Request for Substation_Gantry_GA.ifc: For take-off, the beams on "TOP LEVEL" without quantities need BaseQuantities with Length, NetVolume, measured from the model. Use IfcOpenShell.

First a look at what the model holds.

```python
import ifcopenshell
import ifcopenshell.util.element
import ifcopenshell.util.unit

model = ifcopenshell.open("Substation_Gantry_GA.ifc")
print(model.schema)
for unit_type in ("LENGTHUNIT", "AREAUNIT", "VOLUMEUNIT"):
    print(unit_type, ifcopenshell.util.unit.calculate_unit_scale(model, unit_type))
storey = next(s for s in model.by_type("IfcBuildingStorey") if s.Name == "TOP LEVEL")
beams = [e for e in ifcopenshell.util.element.get_decomposition(storey) if e.is_a("IfcBeam")]
for e in sorted(beams, key=lambda e: e.id()):
    print(e.id(), e.is_a(), e.Name, list(ifcopenshell.util.element.get_psets(e, qtos_only=True)), sep=" | ")
```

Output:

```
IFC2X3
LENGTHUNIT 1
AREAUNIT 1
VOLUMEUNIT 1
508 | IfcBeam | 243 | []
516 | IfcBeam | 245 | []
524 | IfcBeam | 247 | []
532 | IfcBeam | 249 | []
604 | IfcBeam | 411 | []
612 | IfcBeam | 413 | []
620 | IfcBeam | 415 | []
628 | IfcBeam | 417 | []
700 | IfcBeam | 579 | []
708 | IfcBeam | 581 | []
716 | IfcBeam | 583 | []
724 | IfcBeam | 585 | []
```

```python
import ifcopenshell
import ifcopenshell.api.pset
import ifcopenshell.geom
import ifcopenshell.util.element
import ifcopenshell.util.shape
import ifcopenshell.util.unit

model = ifcopenshell.open("Substation_Gantry_GA.ifc")
unit_scale = ifcopenshell.util.unit.calculate_unit_scale(model)
volume_scale = ifcopenshell.util.unit.calculate_unit_scale(model, "VOLUMEUNIT")
settings = ifcopenshell.geom.settings()

storey = next(s for s in model.by_type("IfcBuildingStorey") if s.Name == "TOP LEVEL")
beams = [e for e in ifcopenshell.util.element.get_decomposition(storey) if e.is_a("IfcBeam")]

for e in sorted(beams, key=lambda e: e.id()):
    if ifcopenshell.util.element.get_psets(e, qtos_only=True, should_inherit=False):
        continue
    # Geometry comes back in metres, in the element's own axes.
    shape = ifcopenshell.geom.create_shape(settings, e)
    values = {
        "Length": ifcopenshell.util.shape.get_max_xyz(shape.geometry) / unit_scale,
        "NetVolume": ifcopenshell.util.shape.get_volume(shape.geometry) / volume_scale,
    }
    qto = ifcopenshell.api.pset.add_qto(model, product=e, name="BaseQuantities")
    ifcopenshell.api.pset.edit_qto(model, qto=qto, properties=values)
    print(e.id(), {k: round(v, 3) for k, v in values.items()})

model.write("Substation_Gantry_GA_edited.ifc")
```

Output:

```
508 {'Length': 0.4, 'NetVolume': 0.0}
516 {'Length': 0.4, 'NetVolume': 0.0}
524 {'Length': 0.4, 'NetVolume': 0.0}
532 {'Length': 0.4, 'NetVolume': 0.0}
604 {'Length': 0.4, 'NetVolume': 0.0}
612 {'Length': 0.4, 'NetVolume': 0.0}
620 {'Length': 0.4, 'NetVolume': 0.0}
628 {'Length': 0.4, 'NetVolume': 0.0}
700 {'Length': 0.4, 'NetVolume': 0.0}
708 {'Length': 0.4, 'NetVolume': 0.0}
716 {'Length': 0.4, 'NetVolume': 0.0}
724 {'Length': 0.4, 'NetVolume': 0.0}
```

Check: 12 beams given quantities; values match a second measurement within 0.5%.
